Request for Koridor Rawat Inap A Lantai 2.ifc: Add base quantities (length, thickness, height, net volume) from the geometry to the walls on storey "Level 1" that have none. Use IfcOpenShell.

First a look at what the model holds.

```python
import ifcopenshell
import ifcopenshell.util.element
import ifcopenshell.util.unit

model = ifcopenshell.open("Koridor Rawat Inap A Lantai 2.ifc")
print(model.schema)
for unit_type in ("LENGTHUNIT", "AREAUNIT", "VOLUMEUNIT"):
    print(unit_type, ifcopenshell.util.unit.calculate_unit_scale(model, unit_type))
storey = next(s for s in model.by_type("IfcBuildingStorey") if s.Name == "Level 1")
walls = [e for e in ifcopenshell.util.element.get_decomposition(storey) if e.is_a("IfcWall")]
for e in sorted(walls, key=lambda e: e.id()):
    print(e.id(), e.is_a(), e.Name, list(ifcopenshell.util.element.get_psets(e, qtos_only=True)), sep=" | ")
```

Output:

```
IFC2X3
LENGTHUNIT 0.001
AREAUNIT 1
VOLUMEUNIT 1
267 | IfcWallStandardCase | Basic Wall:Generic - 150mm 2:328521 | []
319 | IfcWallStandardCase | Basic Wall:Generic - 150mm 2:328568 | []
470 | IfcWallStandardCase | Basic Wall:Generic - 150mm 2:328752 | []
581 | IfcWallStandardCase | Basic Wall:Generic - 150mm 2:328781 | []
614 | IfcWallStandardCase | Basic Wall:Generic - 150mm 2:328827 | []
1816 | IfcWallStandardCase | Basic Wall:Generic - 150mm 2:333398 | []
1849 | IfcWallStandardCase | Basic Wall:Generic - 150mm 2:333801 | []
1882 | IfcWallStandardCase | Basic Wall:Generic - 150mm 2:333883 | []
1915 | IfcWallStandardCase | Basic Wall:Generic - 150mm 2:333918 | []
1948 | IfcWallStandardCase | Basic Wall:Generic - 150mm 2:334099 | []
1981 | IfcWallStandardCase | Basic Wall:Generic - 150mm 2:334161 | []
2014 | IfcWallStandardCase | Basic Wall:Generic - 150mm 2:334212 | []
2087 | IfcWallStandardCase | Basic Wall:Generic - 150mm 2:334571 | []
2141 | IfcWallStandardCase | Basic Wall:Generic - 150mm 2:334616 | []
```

```python
import ifcopenshell
import ifcopenshell.api.pset
import ifcopenshell.geom
import ifcopenshell.util.element
import ifcopenshell.util.shape
import ifcopenshell.util.unit

model = ifcopenshell.open("Koridor Rawat Inap A Lantai 2.ifc")
unit_scale = ifcopenshell.util.unit.calculate_unit_scale(model)
volume_scale = ifcopenshell.util.unit.calculate_unit_scale(model, "VOLUMEUNIT")
settings = ifcopenshell.geom.settings()

storey = next(s for s in model.by_type("IfcBuildingStorey") if s.Name == "Level 1")
walls = [e for e in ifcopenshell.util.element.get_decomposition(storey) if e.is_a("IfcWall")]

for e in sorted(walls, key=lambda e: e.id()):
    if ifcopenshell.util.element.get_psets(e, qtos_only=True, should_inherit=False):
        continue
    # Geometry comes back in metres, in the element's own axes.
    shape = ifcopenshell.geom.create_shape(settings, e)
    values = {
        "Length": ifcopenshell.util.shape.get_x(shape.geometry) / unit_scale,
        "Width": ifcopenshell.util.shape.get_y(shape.geometry) / unit_scale,
        "Height": ifcopenshell.util.shape.get_z(shape.geometry) / unit_scale,
        "NetVolume": ifcopenshell.util.shape.get_volume(shape.geometry) / volume_scale,
    }
    qto = ifcopenshell.api.pset.add_qto(model, product=e, name="BaseQuantities")
    ifcopenshell.api.pset.edit_qto(model, qto=qto, properties=values)
    print(e.id(), {k: round(v, 3) for k, v in values.items()})

model.write("Koridor Rawat Inap A Lantai 2_v2.ifc")
```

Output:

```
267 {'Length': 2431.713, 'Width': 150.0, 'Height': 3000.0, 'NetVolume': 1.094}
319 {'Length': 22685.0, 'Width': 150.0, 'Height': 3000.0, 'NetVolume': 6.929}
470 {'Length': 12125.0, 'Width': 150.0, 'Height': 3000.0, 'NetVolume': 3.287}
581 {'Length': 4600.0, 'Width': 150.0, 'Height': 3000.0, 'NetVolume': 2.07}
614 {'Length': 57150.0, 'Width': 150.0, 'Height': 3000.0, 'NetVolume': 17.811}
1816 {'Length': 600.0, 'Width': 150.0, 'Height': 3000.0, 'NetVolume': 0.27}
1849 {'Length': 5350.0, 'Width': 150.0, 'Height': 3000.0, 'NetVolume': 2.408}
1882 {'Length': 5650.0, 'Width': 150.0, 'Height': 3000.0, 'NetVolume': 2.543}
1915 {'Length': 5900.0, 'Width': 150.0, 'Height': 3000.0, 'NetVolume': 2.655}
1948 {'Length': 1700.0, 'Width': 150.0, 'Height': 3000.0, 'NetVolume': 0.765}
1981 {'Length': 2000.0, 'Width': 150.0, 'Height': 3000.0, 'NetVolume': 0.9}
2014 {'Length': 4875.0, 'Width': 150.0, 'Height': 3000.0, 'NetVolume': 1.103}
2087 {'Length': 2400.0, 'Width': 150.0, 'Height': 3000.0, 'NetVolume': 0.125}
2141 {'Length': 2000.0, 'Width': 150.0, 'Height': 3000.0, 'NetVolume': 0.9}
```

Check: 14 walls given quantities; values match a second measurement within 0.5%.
